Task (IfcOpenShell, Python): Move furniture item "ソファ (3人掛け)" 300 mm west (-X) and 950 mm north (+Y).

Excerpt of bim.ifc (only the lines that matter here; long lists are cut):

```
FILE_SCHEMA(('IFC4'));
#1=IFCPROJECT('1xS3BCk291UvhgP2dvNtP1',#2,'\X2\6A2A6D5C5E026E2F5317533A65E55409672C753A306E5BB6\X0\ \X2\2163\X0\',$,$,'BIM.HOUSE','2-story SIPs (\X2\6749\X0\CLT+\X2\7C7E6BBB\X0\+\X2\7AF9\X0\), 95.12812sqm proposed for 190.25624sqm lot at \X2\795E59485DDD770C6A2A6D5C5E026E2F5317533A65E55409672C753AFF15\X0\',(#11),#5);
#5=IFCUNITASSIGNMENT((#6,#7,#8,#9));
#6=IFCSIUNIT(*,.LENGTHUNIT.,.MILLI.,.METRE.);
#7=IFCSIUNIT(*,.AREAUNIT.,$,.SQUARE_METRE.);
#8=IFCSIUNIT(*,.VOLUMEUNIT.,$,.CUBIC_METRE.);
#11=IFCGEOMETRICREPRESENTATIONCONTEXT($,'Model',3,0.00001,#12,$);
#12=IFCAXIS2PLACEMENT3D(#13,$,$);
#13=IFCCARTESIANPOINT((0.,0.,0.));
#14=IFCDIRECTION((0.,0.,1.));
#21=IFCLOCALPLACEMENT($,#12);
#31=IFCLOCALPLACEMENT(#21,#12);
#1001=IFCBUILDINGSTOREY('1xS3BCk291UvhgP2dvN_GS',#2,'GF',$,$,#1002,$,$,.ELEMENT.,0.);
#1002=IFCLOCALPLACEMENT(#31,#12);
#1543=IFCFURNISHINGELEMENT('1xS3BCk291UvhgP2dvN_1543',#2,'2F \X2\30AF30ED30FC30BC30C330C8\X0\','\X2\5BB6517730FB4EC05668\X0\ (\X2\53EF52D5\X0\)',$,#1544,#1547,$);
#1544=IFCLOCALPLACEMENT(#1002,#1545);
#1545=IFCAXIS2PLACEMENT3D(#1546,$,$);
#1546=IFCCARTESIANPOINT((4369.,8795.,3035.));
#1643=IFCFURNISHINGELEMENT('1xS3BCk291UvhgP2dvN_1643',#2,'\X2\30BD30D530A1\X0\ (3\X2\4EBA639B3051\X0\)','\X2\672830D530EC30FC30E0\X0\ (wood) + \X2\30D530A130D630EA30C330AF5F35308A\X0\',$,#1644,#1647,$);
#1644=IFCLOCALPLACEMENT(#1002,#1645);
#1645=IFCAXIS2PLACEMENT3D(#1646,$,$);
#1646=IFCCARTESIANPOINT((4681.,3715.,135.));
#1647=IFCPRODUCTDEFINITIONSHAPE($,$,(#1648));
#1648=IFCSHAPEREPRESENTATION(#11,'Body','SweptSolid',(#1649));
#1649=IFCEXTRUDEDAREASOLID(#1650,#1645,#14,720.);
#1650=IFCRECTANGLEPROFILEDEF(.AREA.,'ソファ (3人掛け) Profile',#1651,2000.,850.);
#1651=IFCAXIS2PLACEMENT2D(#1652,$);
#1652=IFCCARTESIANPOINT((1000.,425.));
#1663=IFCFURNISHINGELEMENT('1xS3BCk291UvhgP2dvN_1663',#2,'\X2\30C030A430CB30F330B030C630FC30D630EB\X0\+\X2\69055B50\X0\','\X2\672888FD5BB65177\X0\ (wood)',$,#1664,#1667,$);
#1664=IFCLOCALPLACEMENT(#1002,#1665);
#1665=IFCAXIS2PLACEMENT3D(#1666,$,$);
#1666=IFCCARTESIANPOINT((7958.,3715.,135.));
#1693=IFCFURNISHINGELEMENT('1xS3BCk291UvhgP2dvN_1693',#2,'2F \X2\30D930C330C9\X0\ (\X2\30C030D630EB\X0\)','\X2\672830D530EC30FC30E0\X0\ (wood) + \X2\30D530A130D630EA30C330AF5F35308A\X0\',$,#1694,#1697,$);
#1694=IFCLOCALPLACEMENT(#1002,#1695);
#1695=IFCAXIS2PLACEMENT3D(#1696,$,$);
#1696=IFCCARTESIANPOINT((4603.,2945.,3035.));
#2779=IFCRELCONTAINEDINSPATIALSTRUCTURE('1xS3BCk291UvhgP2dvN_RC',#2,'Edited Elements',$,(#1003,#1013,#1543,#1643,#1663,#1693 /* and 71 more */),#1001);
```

```python
import ifcopenshell
import ifcopenshell.api.geometry
import ifcopenshell.util.placement

model = ifcopenshell.open("bim.ifc")

item = model.by_id(1643)
matrix = ifcopenshell.util.placement.get_local_placement(item.ObjectPlacement)
matrix[0, 3] -= 300.0
matrix[1, 3] += 950.0
ifcopenshell.api.geometry.edit_object_placement(model, product=item, matrix=matrix, is_si=False)

print(ifcopenshell.util.placement.get_local_placement(item.ObjectPlacement).round(3) + 0.0)

model.write("bim_edited.ifc")
```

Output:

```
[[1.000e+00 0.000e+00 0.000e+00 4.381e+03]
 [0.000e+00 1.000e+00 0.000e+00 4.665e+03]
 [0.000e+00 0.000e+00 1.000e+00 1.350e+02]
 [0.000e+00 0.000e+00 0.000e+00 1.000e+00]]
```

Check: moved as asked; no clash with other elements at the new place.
